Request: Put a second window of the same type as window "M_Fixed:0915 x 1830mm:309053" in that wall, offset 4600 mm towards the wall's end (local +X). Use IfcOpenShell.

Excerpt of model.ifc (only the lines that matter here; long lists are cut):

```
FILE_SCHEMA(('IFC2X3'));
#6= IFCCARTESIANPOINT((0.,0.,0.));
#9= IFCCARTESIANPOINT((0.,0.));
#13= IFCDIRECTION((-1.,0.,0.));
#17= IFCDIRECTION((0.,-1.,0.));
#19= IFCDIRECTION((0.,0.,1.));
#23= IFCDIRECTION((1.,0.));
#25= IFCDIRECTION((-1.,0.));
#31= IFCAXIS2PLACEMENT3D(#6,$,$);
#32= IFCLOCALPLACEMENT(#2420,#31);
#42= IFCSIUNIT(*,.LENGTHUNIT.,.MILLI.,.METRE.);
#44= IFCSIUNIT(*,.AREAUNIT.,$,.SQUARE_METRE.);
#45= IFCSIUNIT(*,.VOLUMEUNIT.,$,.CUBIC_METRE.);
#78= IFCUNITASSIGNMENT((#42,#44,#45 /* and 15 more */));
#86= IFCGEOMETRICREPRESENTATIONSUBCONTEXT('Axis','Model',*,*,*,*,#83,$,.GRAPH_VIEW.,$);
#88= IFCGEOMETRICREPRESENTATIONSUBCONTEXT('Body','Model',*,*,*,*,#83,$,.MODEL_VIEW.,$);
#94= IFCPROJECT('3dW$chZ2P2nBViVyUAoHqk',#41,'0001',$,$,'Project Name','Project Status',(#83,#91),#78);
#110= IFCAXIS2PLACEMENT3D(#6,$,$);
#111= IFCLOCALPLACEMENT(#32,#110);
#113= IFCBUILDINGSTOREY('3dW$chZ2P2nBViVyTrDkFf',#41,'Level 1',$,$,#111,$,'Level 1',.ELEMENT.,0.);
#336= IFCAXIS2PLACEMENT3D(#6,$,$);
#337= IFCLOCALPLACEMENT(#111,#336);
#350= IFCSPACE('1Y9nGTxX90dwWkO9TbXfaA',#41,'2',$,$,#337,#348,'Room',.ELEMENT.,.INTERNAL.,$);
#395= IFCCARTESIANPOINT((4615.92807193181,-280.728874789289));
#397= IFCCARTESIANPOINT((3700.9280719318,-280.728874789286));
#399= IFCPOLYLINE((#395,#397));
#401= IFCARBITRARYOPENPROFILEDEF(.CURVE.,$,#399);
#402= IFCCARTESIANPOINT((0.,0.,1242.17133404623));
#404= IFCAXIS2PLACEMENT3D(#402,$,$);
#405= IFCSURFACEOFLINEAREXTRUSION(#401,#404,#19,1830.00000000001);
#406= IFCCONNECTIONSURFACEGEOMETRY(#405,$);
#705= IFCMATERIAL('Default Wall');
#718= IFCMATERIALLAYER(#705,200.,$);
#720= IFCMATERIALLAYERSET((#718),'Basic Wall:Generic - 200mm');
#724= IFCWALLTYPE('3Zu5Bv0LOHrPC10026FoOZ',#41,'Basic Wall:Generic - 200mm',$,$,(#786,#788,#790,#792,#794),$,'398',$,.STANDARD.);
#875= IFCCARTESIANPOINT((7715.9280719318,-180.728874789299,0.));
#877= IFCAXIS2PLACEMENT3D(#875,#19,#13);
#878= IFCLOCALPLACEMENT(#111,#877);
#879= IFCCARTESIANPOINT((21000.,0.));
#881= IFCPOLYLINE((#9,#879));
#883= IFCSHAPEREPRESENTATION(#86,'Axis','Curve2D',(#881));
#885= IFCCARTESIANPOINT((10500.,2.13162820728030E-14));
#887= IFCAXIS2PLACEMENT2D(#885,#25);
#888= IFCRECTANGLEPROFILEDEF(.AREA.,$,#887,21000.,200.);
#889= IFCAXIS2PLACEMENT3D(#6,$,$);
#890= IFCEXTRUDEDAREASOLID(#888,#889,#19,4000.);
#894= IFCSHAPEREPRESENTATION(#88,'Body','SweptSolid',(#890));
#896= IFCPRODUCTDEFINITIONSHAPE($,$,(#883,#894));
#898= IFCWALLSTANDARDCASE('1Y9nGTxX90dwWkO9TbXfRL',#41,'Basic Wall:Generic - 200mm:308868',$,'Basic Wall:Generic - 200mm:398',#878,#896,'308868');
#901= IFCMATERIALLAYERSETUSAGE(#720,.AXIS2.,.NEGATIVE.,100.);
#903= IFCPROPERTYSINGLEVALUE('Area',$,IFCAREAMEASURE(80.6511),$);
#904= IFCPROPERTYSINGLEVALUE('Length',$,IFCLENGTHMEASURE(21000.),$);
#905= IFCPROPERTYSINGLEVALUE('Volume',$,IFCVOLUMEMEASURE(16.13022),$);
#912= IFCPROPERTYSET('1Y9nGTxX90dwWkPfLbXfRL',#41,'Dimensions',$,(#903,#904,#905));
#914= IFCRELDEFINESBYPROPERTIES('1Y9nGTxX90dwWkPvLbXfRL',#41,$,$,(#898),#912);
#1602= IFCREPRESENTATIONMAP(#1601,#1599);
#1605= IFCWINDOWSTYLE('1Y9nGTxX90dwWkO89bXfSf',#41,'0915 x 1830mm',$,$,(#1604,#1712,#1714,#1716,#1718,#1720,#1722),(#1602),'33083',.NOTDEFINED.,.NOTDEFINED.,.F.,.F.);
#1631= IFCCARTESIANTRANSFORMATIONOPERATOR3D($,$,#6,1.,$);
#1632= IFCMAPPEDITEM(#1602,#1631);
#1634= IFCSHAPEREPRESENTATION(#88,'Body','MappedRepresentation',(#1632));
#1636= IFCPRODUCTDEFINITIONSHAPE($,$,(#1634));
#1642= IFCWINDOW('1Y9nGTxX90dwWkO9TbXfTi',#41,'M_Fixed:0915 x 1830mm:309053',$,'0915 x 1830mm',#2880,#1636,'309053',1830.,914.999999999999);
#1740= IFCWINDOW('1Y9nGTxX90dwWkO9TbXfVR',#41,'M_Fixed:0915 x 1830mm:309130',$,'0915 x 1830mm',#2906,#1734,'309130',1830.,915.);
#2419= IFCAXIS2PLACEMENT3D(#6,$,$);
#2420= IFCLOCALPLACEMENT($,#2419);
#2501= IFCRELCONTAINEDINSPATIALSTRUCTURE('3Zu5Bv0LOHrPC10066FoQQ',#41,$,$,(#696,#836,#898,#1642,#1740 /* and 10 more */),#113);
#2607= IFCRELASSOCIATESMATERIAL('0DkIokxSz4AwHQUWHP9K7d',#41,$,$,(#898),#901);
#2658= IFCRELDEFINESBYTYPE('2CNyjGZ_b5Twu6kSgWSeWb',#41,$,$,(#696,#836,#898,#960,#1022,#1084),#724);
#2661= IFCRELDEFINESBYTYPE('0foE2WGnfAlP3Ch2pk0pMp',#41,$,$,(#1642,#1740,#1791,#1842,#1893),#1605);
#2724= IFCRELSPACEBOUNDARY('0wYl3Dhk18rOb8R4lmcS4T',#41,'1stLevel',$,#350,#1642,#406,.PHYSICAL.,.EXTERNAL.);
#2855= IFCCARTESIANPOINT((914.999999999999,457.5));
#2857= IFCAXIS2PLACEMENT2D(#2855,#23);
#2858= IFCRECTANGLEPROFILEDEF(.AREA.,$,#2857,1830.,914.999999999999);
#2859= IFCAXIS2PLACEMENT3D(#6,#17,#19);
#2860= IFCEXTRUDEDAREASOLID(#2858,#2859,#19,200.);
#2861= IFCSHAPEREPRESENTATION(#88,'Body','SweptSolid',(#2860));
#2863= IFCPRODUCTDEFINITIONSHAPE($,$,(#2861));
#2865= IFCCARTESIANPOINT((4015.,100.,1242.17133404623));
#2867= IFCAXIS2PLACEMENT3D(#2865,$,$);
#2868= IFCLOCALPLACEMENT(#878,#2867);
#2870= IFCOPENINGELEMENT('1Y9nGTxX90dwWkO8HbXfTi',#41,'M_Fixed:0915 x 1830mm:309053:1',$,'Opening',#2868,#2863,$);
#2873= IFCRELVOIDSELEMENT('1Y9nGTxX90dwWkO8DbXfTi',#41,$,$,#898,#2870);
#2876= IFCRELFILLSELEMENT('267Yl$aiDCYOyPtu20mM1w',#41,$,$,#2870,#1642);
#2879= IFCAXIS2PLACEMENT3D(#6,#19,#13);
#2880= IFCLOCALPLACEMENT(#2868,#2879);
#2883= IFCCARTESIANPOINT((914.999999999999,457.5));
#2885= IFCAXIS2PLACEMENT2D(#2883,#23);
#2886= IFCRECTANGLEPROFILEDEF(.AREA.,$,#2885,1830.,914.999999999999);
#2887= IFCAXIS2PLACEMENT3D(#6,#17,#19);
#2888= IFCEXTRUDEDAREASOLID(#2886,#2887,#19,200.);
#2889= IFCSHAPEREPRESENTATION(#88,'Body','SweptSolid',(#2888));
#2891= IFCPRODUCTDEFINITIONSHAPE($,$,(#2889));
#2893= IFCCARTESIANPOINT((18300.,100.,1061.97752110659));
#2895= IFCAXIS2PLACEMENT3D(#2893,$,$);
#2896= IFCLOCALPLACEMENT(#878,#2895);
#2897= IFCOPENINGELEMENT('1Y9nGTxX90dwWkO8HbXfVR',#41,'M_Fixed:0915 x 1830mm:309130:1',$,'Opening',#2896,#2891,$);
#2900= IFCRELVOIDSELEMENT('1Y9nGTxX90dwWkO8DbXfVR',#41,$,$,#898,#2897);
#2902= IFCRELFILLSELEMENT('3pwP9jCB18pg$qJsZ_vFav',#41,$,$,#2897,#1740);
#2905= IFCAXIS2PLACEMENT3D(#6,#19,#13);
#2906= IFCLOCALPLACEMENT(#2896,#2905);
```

```python
import numpy as np
import ifcopenshell
import ifcopenshell.api.feature
import ifcopenshell.api.geometry
import ifcopenshell.api.pset
import ifcopenshell.api.root
import ifcopenshell.geom
import ifcopenshell.util.element
import ifcopenshell.util.placement
import ifcopenshell.util.shape
import ifcopenshell.util.unit

model = ifcopenshell.open("model.ifc")
area_scale = ifcopenshell.util.unit.calculate_unit_scale(model, "AREAUNIT")
volume_scale = ifcopenshell.util.unit.calculate_unit_scale(model, "VOLUMEUNIT")
settings = ifcopenshell.geom.settings()


def volume(element):
    """Net volume in cubic metres, openings subtracted."""
    shape = ifcopenshell.geom.create_shape(settings, element)
    return ifcopenshell.util.shape.get_volume(shape.geometry)


def reuse_history(source, copy):
    """copy_class also copies each property set's owner history, people and application; keep the originals."""
    for rel in copy.IsDefinedBy:
        if rel.is_a("IfcRelDefinesByProperties") and (history := rel.RelatingPropertyDefinition.OwnerHistory):
            rel.RelatingPropertyDefinition.OwnerHistory = source.OwnerHistory
            ifcopenshell.util.element.remove_deep2(model, history)


window = model.by_id(1642)
opening = window.FillsVoids[0].RelatingOpeningElement
wall = opening.VoidsElements[0].RelatingBuildingElement
before = volume(wall)
shift = ifcopenshell.util.placement.get_local_placement(wall.ObjectPlacement)[:3, 0] * 4600.0

# copy_class copies the void relationship, type, container and properties, but no geometry.
new_opening = ifcopenshell.api.root.copy_class(model, product=opening)
new_opening.Representation = ifcopenshell.util.element.copy_deep(
    model, opening.Representation, exclude=["IfcGeometricRepresentationContext", "IfcRepresentationMap"]
)
new_opening.Name = "M_Fixed:0915 x 1830mm"
new_window = ifcopenshell.api.root.copy_class(model, product=window)
new_window.Representation = ifcopenshell.util.element.copy_deep(
    model, window.Representation, exclude=["IfcGeometricRepresentationContext", "IfcRepresentationMap"]
)
new_window.Name = "M_Fixed:0915 x 1830mm"
new_window.Tag = None
reuse_history(window, new_window)
fills = ifcopenshell.api.feature.add_filling(model, opening=new_opening, element=new_window)
fills.OwnerHistory = new_window.OwnerHistory  # required in IFC2X3

for old, new in ((opening, new_opening), (window, new_window)):
    matrix = ifcopenshell.util.placement.get_local_placement(old.ObjectPlacement)
    matrix[:3, 3] += shift
    ifcopenshell.api.geometry.edit_object_placement(model, product=new, matrix=matrix, is_si=False)

# The copied space boundaries still share their surfaces with the original.
for rel in new_window.ProvidesBoundaries:
    if rel.ConnectionGeometry:
        rel.ConnectionGeometry = ifcopenshell.util.element.copy_deep(model, rel.ConnectionGeometry)

# Space boundary surfaces are stored in each space's coordinates; move them too.
for rel in new_window.ProvidesBoundaries:
    if not rel.ConnectionGeometry:
        continue
    surface = rel.ConnectionGeometry.SurfaceOnRelatingElement
    space_matrix = ifcopenshell.util.placement.get_local_placement(rel.RelatingSpace.ObjectPlacement)
    point = np.array(surface.Position.Location.Coordinates) + space_matrix[:3, :3].T @ shift
    surface.Position = model.createIfcAxis2Placement3D(
        model.createIfcCartesianPoint(point.tolist()), surface.Position.Axis, surface.Position.RefDirection
    )

after = volume(wall)
thickness = 0.2  # wall thickness in metres

# Update the wall's stored quantities.
pset = model.by_id(ifcopenshell.util.element.get_pset(wall, "Dimensions", should_inherit=False)["id"])
ifcopenshell.api.pset.edit_pset(model, pset=pset, properties={
    "Area": model.create_entity("IfcAreaMeasure", after / thickness / area_scale),
    "Volume": model.create_entity("IfcVolumeMeasure", after / volume_scale),
})

print(f"wall volume {before:.3f} -> {after:.3f} m3")

model.write("model_updated.ifc")
```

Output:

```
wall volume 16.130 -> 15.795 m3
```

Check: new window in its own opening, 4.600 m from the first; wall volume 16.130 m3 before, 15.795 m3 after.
